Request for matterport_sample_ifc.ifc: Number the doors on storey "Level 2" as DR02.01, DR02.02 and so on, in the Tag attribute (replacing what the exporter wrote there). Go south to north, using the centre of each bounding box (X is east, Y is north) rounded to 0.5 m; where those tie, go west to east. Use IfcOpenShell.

First a look at what the model holds.

```python
import ifcopenshell
import ifcopenshell.util.element
import ifcopenshell.util.placement

model = ifcopenshell.open("matterport_sample_ifc.ifc")
print(model.schema)
storey = next(s for s in model.by_type("IfcBuildingStorey") if s.Name == "Level 2")
doors = [e for e in ifcopenshell.util.element.get_decomposition(storey) if e.is_a("IfcDoor")]
for e in sorted(doors, key=lambda e: e.id()):
    origin = ifcopenshell.util.placement.get_local_placement(e.ObjectPlacement)[:3, 3]
    print(e.id(), e.Tag, e.Name, origin.round(2) + 0.0, sep=" | ")
```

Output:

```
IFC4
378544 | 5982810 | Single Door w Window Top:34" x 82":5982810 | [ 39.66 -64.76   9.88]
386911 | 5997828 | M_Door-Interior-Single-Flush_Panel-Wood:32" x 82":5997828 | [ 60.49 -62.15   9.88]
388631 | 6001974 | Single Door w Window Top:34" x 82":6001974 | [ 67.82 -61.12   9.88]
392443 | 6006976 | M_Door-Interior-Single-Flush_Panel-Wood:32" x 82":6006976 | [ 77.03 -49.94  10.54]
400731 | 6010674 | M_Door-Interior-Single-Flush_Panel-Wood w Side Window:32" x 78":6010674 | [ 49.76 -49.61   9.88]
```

```python
import ifcopenshell
import ifcopenshell.geom
import ifcopenshell.util.element
import ifcopenshell.util.shape

model = ifcopenshell.open("matterport_sample_ifc.ifc")
settings = ifcopenshell.geom.settings()
settings.set("use-world-coords", True)


def centre(element):
    shape = ifcopenshell.geom.create_shape(settings, element)
    return ifcopenshell.util.shape.get_bbox_centroid(shape.geometry)


storey = next(s for s in model.by_type("IfcBuildingStorey") if s.Name == "Level 2")
doors = [e for e in ifcopenshell.util.element.get_decomposition(storey) if e.is_a("IfcDoor")]

# Insertion points can sit at a corner or the storey origin, so sort by the geometry (in metres).
centres = {e: centre(e) for e in doors}
doors.sort(key=lambda e: (round(centres[e][1] / 0.5), centres[e][0]))

for i, e in enumerate(doors, start=1):
    number = f"DR02.{i:02d}"
    e.Tag = number
    print(e.id(), number)

model.write("matterport_sample_ifc_rev.ifc")
```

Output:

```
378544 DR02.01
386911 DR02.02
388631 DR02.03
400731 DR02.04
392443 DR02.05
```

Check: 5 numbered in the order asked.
